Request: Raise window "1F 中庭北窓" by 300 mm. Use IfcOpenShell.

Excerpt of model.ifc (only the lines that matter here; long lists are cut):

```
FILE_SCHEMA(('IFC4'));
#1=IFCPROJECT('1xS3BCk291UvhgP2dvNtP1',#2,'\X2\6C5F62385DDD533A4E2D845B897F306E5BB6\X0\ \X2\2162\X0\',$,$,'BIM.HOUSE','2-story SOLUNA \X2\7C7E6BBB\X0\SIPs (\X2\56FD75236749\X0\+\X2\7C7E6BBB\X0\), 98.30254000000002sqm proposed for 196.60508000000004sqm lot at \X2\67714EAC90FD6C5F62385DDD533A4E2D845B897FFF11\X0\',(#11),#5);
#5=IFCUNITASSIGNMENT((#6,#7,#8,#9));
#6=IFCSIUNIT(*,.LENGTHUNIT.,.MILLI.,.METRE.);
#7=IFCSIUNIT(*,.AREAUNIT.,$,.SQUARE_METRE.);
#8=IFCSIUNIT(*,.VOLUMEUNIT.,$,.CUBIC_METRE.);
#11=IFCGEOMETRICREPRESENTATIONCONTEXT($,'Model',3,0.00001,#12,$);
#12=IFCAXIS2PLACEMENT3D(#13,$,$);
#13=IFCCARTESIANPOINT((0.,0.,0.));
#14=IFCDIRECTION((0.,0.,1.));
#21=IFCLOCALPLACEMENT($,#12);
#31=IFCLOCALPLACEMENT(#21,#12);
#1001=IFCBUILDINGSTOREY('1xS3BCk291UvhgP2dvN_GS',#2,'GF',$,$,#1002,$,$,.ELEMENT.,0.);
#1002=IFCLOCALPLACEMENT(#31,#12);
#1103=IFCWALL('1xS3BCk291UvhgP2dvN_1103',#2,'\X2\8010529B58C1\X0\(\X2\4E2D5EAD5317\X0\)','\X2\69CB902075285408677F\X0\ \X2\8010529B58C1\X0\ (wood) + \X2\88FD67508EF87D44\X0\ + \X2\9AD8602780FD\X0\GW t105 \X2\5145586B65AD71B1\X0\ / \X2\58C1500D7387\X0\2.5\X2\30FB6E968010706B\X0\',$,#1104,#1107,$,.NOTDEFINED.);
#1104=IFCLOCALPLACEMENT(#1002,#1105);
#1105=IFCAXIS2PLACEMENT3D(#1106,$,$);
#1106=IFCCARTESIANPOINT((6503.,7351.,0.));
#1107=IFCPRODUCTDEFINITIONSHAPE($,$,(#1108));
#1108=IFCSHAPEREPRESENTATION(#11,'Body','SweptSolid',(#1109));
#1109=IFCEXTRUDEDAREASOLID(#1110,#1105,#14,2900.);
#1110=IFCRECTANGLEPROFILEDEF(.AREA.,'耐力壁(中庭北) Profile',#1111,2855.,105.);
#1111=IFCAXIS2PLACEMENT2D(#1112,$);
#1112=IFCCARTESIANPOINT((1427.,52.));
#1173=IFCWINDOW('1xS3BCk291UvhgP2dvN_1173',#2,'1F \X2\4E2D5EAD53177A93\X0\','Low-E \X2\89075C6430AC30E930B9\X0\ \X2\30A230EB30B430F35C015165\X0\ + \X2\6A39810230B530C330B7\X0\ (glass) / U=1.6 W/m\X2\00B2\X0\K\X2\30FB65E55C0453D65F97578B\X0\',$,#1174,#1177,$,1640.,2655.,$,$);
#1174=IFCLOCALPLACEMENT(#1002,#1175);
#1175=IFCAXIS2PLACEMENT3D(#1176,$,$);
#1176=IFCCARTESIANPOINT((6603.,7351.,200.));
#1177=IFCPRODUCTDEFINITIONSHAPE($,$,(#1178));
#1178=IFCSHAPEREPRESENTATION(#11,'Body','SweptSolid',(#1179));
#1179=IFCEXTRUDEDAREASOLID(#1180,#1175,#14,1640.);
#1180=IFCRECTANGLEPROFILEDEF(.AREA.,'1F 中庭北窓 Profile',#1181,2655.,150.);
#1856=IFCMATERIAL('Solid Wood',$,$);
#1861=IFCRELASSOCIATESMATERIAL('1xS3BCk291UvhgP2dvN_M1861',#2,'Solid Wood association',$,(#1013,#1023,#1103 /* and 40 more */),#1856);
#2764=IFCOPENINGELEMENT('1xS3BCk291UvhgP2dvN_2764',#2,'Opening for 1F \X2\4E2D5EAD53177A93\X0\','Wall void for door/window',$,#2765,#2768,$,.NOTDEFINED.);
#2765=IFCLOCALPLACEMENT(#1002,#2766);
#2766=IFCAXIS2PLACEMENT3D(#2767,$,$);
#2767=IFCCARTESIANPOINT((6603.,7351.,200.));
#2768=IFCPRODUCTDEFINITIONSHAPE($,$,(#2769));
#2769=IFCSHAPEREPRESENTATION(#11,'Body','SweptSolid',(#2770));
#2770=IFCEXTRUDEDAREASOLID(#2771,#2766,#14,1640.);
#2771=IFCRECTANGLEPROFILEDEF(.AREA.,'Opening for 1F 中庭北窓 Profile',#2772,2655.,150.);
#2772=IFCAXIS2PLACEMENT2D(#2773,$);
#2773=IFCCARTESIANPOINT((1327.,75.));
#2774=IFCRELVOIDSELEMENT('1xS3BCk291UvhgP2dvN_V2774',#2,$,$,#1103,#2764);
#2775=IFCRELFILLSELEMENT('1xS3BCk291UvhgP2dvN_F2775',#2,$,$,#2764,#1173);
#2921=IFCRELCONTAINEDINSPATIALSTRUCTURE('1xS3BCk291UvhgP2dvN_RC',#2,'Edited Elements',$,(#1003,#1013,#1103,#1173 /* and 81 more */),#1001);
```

```python
import numpy as np
import ifcopenshell
import ifcopenshell.api.geometry
import ifcopenshell.util.placement
import ifcopenshell.util.unit

model = ifcopenshell.open("model.ifc")
unit_scale = ifcopenshell.util.unit.calculate_unit_scale(model)

window = model.by_guid("1xS3BCk291UvhgP2dvN_1173")
opening = window.FillsVoids[0].RelatingOpeningElement
dz = 300.0

shift = np.array([0.0, 0.0, dz])
# The window is not placed relative to its opening, so move both.
for product in (opening, window):
    matrix = ifcopenshell.util.placement.get_local_placement(product.ObjectPlacement)
    matrix[:3, 3] += shift
    ifcopenshell.api.geometry.edit_object_placement(model, product=product, matrix=matrix, is_si=False)

print(f"moved by {dz * unit_scale:+.3f} m")

model.write("model-out.ifc")
```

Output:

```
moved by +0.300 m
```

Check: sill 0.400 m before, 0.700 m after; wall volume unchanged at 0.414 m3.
